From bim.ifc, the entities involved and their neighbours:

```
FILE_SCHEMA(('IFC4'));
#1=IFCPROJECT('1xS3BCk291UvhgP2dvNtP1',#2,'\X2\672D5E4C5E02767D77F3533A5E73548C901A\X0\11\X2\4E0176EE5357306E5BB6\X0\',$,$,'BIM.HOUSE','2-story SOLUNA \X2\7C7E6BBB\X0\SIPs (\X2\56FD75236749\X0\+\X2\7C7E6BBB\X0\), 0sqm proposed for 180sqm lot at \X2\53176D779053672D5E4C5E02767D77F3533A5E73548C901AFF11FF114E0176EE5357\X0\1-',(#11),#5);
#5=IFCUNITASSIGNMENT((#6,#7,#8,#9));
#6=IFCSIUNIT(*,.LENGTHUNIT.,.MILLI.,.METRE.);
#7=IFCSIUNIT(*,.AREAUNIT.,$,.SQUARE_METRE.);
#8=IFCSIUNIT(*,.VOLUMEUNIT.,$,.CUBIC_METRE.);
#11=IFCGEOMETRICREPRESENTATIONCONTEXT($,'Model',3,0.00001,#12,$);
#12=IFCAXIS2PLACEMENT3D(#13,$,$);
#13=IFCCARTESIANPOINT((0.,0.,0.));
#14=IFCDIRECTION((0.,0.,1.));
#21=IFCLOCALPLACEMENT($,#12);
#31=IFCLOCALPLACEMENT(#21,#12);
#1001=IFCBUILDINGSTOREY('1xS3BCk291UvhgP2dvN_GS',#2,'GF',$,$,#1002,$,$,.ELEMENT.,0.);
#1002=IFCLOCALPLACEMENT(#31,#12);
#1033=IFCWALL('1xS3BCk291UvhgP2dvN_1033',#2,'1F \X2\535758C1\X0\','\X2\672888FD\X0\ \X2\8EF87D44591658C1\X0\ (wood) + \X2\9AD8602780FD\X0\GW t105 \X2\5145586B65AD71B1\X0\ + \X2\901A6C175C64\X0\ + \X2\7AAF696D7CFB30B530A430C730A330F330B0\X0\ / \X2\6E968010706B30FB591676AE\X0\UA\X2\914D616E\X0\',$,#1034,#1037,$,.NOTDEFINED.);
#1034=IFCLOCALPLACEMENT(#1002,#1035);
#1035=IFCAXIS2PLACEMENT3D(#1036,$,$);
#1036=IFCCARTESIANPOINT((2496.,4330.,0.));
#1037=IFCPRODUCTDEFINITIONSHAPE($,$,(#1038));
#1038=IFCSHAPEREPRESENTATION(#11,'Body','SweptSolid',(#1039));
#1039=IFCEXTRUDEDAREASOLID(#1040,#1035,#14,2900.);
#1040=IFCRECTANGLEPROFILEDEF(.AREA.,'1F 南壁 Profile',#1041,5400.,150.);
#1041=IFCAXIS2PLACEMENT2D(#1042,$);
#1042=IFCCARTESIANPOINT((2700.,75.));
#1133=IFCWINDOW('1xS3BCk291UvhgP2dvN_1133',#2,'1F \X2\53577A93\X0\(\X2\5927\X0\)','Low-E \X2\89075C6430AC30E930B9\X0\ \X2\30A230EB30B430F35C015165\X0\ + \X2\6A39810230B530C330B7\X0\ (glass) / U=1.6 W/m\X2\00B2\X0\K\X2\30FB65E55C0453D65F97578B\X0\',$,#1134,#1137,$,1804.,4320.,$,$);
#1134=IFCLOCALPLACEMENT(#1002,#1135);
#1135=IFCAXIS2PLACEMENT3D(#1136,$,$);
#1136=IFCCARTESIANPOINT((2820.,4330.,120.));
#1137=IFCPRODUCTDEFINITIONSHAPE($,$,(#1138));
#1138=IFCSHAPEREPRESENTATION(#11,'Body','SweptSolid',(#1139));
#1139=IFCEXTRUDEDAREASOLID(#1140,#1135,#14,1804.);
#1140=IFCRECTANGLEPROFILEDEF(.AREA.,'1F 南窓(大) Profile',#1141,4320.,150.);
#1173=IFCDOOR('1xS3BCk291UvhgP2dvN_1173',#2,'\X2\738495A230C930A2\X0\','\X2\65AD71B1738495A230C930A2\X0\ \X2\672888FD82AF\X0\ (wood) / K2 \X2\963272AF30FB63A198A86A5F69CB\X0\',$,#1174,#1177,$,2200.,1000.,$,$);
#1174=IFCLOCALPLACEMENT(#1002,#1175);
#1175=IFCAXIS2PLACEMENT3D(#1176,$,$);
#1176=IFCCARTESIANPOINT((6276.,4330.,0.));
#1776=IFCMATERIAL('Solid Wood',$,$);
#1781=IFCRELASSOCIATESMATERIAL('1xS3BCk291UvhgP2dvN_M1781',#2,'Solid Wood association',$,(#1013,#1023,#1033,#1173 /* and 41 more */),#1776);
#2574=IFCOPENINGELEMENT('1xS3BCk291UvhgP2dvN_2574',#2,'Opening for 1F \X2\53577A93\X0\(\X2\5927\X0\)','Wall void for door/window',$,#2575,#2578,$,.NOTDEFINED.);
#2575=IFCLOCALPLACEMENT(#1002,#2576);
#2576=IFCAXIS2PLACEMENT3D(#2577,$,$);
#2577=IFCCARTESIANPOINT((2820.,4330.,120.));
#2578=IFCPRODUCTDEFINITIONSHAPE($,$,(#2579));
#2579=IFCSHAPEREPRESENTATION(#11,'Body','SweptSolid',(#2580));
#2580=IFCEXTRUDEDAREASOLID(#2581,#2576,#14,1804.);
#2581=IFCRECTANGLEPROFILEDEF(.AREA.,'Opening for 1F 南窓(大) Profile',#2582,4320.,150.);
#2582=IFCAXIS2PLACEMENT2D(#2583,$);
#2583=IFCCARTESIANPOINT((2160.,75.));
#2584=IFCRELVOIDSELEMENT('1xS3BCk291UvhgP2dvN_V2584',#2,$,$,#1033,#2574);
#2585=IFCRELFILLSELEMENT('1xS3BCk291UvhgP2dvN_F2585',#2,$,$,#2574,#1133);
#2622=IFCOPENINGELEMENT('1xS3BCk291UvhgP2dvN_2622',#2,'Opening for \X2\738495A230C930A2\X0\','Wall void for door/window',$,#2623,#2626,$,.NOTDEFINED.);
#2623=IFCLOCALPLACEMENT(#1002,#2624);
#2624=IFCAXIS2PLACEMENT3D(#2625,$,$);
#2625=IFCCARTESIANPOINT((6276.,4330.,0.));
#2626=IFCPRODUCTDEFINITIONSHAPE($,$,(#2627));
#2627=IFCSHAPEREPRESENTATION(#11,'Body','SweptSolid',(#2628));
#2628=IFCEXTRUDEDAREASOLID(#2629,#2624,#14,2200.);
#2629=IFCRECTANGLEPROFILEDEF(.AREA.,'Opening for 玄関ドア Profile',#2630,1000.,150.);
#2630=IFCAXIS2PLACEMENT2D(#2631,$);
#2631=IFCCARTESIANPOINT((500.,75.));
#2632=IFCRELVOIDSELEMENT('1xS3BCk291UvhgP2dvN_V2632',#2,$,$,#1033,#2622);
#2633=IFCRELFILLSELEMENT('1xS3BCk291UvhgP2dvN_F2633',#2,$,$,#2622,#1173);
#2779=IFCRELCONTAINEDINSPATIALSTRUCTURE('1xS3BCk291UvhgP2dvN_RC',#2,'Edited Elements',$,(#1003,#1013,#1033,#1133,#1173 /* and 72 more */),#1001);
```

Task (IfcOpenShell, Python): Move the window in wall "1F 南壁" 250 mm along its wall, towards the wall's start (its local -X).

```python
import ifcopenshell
import ifcopenshell.api.geometry
import ifcopenshell.util.placement
import ifcopenshell.util.unit

model = ifcopenshell.open("bim.ifc")
unit_scale = ifcopenshell.util.unit.calculate_unit_scale(model)

window = model.by_guid("1xS3BCk291UvhgP2dvN_1133")
opening = window.FillsVoids[0].RelatingOpeningElement
wall = opening.VoidsElements[0].RelatingBuildingElement

wall_matrix = ifcopenshell.util.placement.get_local_placement(wall.ObjectPlacement)
shift = wall_matrix[:3, 0] * -0.25 / unit_scale
before = ifcopenshell.util.placement.get_local_placement(window.ObjectPlacement)[:3, 3].copy()

# The window is not placed relative to its opening, so move both.
for product in (opening, window):
    matrix = ifcopenshell.util.placement.get_local_placement(product.ObjectPlacement)
    matrix[:3, 3] += shift
    ifcopenshell.api.geometry.edit_object_placement(model, product=product, matrix=matrix, is_si=False)

after = ifcopenshell.util.placement.get_local_placement(window.ObjectPlacement)[:3, 3]
print("window moved by", (after - before).round(3) + 0.0)

model.write("bim_edited.ifc")
```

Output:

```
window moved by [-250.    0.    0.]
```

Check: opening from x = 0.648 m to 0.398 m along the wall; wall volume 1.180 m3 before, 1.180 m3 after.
